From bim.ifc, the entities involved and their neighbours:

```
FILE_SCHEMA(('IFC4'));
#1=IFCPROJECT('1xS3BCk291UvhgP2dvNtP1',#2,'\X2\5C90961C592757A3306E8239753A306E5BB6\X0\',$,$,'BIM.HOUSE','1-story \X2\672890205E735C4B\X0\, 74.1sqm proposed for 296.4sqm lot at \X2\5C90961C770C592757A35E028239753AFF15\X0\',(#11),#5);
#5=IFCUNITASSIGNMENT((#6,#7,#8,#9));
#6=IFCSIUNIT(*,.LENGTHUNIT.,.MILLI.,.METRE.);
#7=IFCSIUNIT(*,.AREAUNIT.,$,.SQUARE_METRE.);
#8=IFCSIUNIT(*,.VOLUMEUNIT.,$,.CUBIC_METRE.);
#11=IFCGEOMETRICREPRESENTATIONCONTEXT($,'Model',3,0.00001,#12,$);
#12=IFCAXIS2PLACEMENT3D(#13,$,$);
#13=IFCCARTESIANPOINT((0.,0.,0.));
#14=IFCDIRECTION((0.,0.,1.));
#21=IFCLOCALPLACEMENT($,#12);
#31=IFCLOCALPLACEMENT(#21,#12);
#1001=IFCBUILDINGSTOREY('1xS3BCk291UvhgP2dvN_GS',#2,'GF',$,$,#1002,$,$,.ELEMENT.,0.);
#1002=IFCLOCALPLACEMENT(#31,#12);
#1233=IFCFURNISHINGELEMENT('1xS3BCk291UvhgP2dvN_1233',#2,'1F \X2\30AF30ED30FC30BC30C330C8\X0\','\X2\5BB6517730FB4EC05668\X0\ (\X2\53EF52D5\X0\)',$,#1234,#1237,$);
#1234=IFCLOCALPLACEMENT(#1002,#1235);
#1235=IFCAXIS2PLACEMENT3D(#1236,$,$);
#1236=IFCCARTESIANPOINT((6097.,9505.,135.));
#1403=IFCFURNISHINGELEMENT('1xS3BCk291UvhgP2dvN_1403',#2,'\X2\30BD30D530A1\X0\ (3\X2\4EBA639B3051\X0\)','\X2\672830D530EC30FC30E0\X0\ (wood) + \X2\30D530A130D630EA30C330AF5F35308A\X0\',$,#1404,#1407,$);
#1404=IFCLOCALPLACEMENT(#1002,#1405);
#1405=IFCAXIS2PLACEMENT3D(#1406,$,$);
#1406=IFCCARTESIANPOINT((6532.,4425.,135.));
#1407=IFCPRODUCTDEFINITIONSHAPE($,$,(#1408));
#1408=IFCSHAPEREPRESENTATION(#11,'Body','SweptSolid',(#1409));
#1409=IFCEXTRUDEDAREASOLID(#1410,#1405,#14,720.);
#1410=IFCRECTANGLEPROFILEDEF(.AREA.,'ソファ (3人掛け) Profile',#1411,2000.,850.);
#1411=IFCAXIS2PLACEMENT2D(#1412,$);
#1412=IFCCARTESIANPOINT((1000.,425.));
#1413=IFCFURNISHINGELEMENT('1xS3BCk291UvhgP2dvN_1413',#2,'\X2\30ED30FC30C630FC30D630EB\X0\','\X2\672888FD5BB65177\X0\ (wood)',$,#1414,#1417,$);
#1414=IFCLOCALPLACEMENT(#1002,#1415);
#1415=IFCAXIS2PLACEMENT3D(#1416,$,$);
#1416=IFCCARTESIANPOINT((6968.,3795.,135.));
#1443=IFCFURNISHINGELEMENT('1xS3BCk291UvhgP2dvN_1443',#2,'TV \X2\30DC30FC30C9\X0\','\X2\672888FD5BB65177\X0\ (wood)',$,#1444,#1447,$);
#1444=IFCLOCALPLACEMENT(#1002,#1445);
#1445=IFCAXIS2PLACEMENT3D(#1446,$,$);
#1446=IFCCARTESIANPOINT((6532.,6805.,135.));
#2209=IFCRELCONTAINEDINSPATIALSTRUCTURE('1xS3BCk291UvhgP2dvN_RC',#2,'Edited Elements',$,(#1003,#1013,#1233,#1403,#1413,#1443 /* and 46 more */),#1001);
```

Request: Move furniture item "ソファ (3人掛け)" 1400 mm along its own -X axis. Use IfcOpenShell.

```python
import ifcopenshell
import ifcopenshell.api.geometry
import ifcopenshell.util.placement
import ifcopenshell.util.unit

model = ifcopenshell.open("bim.ifc")
unit_scale = ifcopenshell.util.unit.calculate_unit_scale(model)

item = model.by_guid("1xS3BCk291UvhgP2dvN_1403")
matrix = ifcopenshell.util.placement.get_local_placement(item.ObjectPlacement)
matrix[:3, 3] -= matrix[:3, 0] * 1.4 / unit_scale
ifcopenshell.api.geometry.edit_object_placement(model, product=item, matrix=matrix, is_si=False)

print(ifcopenshell.util.placement.get_local_placement(item.ObjectPlacement).round(3) + 0.0)

model.write("bim_updated.ifc")
```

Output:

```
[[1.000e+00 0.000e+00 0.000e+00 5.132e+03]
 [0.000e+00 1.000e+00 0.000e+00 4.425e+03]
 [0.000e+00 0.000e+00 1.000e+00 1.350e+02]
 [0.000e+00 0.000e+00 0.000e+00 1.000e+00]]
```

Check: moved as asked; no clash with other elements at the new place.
